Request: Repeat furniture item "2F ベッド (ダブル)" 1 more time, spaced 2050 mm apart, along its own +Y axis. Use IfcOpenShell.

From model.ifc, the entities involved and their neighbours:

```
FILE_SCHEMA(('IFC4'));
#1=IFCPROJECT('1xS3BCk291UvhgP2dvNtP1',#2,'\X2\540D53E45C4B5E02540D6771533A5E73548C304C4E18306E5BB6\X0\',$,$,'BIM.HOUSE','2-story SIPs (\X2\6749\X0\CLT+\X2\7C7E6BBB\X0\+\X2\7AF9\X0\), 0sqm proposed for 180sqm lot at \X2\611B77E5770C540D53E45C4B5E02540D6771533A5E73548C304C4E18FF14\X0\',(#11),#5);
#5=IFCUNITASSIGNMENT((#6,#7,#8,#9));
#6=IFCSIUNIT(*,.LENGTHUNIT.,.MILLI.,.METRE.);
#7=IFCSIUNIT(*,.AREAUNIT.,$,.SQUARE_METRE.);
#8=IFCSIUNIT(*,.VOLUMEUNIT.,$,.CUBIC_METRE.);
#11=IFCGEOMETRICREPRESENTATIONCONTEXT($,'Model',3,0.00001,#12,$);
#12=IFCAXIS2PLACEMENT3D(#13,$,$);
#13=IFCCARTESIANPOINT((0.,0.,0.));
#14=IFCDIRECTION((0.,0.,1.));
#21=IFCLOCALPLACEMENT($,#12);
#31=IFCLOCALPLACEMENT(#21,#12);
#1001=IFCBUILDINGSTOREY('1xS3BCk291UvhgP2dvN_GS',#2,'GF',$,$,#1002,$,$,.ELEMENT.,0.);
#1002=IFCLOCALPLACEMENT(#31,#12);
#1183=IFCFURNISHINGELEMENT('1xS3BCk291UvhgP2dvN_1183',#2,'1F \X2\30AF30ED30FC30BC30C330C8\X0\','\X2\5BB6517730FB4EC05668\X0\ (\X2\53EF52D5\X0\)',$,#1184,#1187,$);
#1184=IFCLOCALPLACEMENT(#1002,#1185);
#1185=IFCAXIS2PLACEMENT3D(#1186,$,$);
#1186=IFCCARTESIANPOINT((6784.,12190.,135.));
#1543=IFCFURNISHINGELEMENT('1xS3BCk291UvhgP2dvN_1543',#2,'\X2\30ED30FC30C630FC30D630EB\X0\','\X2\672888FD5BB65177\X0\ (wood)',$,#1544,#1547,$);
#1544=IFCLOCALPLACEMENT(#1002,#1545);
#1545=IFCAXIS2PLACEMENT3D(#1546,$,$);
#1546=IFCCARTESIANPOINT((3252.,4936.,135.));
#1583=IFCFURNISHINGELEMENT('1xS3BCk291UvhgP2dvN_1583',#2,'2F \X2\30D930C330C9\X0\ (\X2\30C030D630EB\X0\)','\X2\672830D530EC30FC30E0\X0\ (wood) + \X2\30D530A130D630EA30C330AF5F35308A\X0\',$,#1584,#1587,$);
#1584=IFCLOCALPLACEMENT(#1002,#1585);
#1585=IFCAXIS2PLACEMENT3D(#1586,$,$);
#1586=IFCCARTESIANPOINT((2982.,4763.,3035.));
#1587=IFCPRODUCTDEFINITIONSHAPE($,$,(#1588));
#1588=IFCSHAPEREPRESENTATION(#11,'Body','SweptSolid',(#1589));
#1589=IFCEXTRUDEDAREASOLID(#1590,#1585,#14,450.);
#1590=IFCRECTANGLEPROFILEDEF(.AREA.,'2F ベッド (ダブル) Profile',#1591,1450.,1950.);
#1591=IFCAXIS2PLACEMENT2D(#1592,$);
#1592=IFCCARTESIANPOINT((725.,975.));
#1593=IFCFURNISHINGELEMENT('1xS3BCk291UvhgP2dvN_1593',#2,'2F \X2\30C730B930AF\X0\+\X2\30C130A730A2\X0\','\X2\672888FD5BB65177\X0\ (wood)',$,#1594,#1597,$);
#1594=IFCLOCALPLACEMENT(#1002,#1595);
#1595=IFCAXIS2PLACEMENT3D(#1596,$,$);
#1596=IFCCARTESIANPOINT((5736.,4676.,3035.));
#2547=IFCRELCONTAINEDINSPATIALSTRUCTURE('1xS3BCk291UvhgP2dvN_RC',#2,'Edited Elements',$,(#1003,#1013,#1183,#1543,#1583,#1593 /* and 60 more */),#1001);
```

```python
import ifcopenshell
import ifcopenshell.api.geometry
import ifcopenshell.api.root
import ifcopenshell.util.element
import ifcopenshell.util.placement
import ifcopenshell.util.unit

model = ifcopenshell.open("model.ifc")
unit_scale = ifcopenshell.util.unit.calculate_unit_scale(model)


def reuse_history(source, copy):
    """copy_class also copies each property set's owner history, people and application; keep the originals."""
    for rel in copy.IsDefinedBy:
        if rel.is_a("IfcRelDefinesByProperties") and (history := rel.RelatingPropertyDefinition.OwnerHistory):
            rel.RelatingPropertyDefinition.OwnerHistory = source.OwnerHistory
            ifcopenshell.util.element.remove_deep2(model, history)


source = model.by_guid("1xS3BCk291UvhgP2dvN_1583")
base = ifcopenshell.util.placement.get_local_placement(source.ObjectPlacement)
step = base[:3, 1] * 2.05 / unit_scale

for i in range(1, 2):
    copy = ifcopenshell.api.root.copy_class(model, product=source)
    copy.Representation = ifcopenshell.util.element.copy_deep(
        model, source.Representation, exclude=["IfcGeometricRepresentationContext", "IfcRepresentationMap"]
    )
    reuse_history(source, copy)
    matrix = base.copy()
    matrix[:3, 3] += i * step
    print("added at", matrix[:3, 3].round(3) + 0.0)
    ifcopenshell.api.geometry.edit_object_placement(model, product=copy, matrix=matrix, is_si=False)

model.write("model-out.ifc")
```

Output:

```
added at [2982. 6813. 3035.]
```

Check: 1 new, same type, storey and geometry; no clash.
